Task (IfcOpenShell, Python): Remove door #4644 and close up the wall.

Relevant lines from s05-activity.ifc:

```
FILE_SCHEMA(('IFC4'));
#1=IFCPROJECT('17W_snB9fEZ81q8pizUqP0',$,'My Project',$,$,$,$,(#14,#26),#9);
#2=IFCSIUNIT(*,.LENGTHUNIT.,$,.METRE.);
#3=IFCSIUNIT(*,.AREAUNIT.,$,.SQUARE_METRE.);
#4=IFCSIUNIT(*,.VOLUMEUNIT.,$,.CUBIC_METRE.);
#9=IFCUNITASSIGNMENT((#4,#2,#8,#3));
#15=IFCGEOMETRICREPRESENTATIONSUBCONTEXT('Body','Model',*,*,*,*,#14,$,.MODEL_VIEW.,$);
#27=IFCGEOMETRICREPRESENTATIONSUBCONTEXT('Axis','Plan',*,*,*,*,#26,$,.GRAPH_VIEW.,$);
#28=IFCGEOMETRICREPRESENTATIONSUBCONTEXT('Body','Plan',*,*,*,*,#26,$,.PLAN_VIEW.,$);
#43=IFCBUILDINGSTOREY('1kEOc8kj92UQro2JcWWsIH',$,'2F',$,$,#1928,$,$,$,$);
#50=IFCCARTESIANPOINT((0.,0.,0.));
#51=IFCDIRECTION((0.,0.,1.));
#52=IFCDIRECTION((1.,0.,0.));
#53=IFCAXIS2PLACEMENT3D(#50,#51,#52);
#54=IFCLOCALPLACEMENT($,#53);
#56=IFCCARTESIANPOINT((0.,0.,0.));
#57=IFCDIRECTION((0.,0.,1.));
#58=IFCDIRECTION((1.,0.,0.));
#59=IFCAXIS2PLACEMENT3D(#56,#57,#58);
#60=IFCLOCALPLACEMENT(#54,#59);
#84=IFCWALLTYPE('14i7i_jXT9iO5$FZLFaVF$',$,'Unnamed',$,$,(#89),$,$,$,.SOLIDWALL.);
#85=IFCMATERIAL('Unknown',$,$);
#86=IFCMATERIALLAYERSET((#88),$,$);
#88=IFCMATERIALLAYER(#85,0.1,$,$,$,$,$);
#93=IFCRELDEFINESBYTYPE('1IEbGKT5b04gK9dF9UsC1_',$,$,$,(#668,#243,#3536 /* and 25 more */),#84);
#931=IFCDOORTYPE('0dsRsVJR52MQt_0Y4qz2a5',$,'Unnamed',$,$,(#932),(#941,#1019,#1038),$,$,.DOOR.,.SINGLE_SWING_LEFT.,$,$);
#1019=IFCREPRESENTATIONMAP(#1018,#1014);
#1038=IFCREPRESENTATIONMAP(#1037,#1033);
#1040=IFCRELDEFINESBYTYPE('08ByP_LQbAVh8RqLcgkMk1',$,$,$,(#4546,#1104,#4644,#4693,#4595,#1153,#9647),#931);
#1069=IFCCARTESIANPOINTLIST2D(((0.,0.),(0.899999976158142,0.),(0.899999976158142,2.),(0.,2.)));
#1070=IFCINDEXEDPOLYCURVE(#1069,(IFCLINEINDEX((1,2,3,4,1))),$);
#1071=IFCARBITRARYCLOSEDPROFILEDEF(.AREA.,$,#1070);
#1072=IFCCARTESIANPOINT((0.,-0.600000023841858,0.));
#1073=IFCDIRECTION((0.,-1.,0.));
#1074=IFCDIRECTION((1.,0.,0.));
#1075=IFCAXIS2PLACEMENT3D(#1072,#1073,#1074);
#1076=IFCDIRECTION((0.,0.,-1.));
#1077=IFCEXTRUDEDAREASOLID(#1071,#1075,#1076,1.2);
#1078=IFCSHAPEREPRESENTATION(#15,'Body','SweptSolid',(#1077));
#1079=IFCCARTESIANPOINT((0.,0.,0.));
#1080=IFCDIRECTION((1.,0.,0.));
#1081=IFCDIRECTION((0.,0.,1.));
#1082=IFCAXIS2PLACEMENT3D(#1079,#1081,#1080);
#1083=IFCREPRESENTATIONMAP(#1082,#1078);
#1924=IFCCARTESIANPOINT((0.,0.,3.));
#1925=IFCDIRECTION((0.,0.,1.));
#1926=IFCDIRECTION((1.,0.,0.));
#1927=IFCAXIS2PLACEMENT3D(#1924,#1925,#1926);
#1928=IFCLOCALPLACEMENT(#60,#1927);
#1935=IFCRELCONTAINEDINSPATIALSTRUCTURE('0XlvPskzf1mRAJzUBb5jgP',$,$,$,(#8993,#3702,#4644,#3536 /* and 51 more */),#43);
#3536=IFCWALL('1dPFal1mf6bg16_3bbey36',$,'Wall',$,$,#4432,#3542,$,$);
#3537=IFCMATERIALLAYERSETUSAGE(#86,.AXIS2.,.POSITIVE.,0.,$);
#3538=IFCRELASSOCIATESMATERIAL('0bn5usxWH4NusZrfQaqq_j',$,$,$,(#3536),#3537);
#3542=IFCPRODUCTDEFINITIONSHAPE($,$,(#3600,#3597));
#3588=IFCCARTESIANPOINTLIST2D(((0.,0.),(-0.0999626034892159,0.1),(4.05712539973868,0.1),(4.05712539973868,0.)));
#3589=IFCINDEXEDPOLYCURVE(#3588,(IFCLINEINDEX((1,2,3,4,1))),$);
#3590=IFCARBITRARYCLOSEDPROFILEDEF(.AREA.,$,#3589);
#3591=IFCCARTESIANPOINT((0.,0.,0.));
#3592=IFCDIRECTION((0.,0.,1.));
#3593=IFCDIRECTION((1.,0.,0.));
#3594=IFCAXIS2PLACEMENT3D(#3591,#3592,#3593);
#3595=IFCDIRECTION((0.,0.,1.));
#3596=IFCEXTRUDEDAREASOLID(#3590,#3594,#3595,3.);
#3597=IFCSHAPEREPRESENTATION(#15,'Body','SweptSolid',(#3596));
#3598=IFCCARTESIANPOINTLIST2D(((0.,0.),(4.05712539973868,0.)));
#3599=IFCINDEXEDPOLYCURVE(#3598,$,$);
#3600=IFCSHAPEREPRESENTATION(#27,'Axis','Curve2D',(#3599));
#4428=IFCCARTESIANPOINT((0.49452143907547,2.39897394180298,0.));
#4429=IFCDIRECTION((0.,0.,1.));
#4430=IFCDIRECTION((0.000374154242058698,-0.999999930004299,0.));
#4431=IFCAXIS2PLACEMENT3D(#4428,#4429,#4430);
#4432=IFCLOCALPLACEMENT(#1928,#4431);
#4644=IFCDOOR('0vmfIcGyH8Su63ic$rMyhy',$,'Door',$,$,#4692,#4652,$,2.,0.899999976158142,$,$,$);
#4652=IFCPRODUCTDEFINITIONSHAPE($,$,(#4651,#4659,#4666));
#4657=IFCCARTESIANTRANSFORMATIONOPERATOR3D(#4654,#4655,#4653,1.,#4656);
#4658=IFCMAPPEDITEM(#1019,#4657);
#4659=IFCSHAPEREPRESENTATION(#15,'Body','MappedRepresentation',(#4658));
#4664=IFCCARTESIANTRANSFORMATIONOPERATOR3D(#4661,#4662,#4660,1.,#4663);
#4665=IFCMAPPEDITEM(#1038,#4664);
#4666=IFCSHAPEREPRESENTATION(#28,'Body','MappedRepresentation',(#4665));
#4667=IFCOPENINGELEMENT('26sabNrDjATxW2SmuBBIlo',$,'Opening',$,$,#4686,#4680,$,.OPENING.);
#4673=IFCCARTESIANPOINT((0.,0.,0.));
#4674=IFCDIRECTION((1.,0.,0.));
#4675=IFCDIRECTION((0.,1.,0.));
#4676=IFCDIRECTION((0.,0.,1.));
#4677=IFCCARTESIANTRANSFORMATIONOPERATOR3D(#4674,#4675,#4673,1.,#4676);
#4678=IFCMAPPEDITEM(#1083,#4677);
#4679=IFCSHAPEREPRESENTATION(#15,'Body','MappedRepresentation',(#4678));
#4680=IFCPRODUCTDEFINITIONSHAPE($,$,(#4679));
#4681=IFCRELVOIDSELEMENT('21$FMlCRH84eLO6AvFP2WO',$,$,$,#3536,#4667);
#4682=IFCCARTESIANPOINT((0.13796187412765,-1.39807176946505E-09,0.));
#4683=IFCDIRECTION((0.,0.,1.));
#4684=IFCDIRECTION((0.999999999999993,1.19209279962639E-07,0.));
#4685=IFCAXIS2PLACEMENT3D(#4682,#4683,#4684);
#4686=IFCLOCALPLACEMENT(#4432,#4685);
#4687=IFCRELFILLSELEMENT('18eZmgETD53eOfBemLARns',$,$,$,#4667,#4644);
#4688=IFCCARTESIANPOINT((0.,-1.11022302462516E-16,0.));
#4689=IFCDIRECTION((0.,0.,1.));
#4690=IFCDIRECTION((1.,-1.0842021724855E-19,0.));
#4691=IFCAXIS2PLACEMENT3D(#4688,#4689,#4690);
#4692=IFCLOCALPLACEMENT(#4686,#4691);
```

```python
import ifcopenshell
import ifcopenshell.api.feature
import ifcopenshell.api.root
import ifcopenshell.geom
import ifcopenshell.util.shape

model = ifcopenshell.open("s05-activity.ifc")
settings = ifcopenshell.geom.settings()


def volume(element):
    """Net volume in cubic metres, openings subtracted."""
    shape = ifcopenshell.geom.create_shape(settings, element)
    return ifcopenshell.util.shape.get_volume(shape.geometry)


door = model.by_guid("0vmfIcGyH8Su63ic$rMyhy")
opening = door.FillsVoids[0].RelatingOpeningElement
wall = opening.VoidsElements[0].RelatingBuildingElement
before = volume(wall)

ifcopenshell.api.root.remove_product(model, product=door)
ifcopenshell.api.feature.remove_feature(model, feature=opening)

after = volume(wall)

print(f"wall volume {before:.3f} -> {after:.3f} m3")

model.write("s05-activity_edited.ifc")
```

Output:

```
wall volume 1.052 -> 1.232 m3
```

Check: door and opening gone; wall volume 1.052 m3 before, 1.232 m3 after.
